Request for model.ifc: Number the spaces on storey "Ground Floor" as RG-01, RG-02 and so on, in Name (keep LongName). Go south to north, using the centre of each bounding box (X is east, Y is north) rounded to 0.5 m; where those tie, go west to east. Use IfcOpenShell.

First a look at what the model holds.

```python
import ifcopenshell
import ifcopenshell.util.element
import ifcopenshell.util.placement

model = ifcopenshell.open("model.ifc")
print(model.schema)
storey = next(s for s in model.by_type("IfcBuildingStorey") if s.Name == "Ground Floor")
spaces = [e for e in ifcopenshell.util.element.get_decomposition(storey) if e.is_a("IfcSpace")]
for e in sorted(spaces, key=lambda e: e.id()):
    origin = ifcopenshell.util.placement.get_local_placement(e.ObjectPlacement)[:3, 3]
    print(e.id(), e.Name, e.LongName, origin.round(2) + 0.0, sep=" | ")
```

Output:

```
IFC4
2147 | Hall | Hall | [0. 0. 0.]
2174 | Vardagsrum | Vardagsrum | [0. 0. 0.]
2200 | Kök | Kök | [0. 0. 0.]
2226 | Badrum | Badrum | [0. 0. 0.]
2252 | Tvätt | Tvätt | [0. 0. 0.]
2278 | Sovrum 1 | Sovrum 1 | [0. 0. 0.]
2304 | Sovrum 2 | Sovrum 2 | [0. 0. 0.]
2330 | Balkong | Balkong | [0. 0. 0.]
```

```python
import ifcopenshell
import ifcopenshell.geom
import ifcopenshell.util.element
import ifcopenshell.util.shape

model = ifcopenshell.open("model.ifc")
settings = ifcopenshell.geom.settings()
settings.set("use-world-coords", True)


def centre(element):
    shape = ifcopenshell.geom.create_shape(settings, element)
    return ifcopenshell.util.shape.get_bbox_centroid(shape.geometry)


storey = next(s for s in model.by_type("IfcBuildingStorey") if s.Name == "Ground Floor")
spaces = [e for e in ifcopenshell.util.element.get_decomposition(storey) if e.is_a("IfcSpace")]

# Insertion points can sit at a corner or the storey origin, so sort by the geometry (in metres).
centres = {e: centre(e) for e in spaces}
spaces.sort(key=lambda e: (round(centres[e][1] / 0.5), centres[e][0]))

for i, e in enumerate(spaces, start=1):
    number = f"RG-{i:02d}"
    e.Name = number
    print(e.id(), number)

model.write("model_rev.ifc")
```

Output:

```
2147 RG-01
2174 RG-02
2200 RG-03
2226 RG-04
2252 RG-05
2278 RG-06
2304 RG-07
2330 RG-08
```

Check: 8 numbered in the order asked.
